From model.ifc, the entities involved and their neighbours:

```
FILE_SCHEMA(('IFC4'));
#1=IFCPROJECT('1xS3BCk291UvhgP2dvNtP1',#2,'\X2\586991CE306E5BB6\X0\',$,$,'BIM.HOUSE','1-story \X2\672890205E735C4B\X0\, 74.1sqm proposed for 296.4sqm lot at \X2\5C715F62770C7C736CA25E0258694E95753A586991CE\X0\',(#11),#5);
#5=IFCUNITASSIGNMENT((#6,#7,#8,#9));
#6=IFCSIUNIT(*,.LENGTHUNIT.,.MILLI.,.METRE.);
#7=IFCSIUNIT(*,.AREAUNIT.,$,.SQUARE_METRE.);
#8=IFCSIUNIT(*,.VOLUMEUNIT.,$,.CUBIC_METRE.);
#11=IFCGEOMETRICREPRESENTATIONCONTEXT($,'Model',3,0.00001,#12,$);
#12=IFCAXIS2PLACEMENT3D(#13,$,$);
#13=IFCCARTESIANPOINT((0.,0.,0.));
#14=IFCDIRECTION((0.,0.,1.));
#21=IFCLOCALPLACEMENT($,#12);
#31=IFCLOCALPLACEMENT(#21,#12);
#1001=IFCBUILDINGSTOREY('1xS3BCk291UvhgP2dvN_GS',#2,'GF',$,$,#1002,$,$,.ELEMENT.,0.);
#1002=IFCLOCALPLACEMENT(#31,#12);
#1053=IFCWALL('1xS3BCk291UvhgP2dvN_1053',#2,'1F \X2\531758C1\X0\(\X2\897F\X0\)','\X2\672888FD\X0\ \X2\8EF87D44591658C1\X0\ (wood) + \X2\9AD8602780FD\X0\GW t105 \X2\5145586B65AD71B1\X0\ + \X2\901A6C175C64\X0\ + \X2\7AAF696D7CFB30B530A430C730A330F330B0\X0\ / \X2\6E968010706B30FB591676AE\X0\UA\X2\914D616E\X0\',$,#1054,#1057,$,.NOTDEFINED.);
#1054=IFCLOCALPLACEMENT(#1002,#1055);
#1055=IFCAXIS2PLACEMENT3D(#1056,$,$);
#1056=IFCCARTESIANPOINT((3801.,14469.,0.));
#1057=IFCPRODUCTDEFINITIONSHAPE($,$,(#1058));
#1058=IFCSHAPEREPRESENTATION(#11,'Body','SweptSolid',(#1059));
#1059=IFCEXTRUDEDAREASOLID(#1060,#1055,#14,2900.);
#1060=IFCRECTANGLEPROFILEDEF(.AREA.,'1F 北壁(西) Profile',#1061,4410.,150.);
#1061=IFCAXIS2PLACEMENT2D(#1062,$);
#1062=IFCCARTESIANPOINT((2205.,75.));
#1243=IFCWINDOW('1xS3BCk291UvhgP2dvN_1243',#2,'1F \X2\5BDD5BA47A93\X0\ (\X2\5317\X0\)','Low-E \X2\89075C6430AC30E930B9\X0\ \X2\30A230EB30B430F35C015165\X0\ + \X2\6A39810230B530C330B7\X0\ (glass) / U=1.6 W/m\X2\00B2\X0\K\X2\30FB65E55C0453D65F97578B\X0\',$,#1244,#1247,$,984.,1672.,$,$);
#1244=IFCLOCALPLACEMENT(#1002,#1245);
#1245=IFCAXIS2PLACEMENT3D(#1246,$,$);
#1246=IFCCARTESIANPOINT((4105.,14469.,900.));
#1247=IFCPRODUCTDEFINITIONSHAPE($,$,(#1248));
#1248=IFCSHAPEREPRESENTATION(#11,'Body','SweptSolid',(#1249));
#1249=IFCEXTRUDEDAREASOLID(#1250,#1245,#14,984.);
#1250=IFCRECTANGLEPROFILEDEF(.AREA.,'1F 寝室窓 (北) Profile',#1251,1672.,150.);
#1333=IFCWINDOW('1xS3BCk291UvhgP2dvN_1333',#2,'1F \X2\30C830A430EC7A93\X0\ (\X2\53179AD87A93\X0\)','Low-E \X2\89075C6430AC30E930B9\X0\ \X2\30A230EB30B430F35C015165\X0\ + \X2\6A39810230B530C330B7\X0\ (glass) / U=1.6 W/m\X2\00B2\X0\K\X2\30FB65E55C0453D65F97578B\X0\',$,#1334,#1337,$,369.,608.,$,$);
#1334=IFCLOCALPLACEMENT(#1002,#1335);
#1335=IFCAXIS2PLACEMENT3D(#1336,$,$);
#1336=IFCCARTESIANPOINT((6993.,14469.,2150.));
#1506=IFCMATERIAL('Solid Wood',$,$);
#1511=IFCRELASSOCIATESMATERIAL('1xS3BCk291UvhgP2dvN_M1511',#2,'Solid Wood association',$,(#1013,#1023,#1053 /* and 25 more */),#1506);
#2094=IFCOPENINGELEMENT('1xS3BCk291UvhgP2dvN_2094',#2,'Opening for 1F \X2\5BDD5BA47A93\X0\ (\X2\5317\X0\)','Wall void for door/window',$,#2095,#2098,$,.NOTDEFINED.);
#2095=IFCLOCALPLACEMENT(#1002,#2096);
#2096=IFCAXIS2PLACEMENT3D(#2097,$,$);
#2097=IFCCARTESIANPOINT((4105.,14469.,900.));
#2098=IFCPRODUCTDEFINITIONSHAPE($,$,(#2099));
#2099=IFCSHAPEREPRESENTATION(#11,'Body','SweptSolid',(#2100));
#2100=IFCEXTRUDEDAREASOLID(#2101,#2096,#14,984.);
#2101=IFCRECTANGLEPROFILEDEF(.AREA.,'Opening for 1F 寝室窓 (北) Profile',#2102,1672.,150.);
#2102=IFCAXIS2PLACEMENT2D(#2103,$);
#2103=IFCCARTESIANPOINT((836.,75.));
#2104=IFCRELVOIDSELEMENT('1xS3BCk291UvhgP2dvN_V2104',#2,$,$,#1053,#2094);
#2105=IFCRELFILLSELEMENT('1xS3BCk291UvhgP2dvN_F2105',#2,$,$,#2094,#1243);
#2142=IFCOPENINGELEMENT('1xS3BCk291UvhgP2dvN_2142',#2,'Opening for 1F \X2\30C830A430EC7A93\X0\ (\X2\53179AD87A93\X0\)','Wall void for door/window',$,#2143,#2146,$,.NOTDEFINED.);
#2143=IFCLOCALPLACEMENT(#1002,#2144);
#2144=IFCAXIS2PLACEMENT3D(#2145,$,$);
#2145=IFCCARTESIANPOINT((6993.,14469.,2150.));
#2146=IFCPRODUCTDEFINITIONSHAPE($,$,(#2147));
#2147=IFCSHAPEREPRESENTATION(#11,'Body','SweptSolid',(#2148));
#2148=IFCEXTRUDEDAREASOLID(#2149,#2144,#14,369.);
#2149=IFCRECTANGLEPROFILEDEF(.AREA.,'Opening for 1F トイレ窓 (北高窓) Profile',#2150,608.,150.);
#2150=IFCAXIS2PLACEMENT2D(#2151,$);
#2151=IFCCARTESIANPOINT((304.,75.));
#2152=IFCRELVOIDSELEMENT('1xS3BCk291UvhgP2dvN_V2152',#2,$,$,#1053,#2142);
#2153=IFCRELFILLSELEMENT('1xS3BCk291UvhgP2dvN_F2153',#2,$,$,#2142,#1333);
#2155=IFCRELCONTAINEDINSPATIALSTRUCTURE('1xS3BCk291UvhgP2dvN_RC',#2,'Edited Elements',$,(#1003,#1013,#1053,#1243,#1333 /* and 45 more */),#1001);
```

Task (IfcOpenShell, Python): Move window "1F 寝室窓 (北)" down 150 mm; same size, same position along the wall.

```python
import numpy as np
import ifcopenshell
import ifcopenshell.api.geometry
import ifcopenshell.util.placement
import ifcopenshell.util.unit

model = ifcopenshell.open("model.ifc")
unit_scale = ifcopenshell.util.unit.calculate_unit_scale(model)

window = model.by_guid("1xS3BCk291UvhgP2dvN_1243")
opening = window.FillsVoids[0].RelatingOpeningElement
dz = -0.15 / unit_scale

shift = np.array([0.0, 0.0, dz])
# The window is not placed relative to its opening, so move both.
for product in (opening, window):
    matrix = ifcopenshell.util.placement.get_local_placement(product.ObjectPlacement)
    matrix[:3, 3] += shift
    ifcopenshell.api.geometry.edit_object_placement(model, product=product, matrix=matrix, is_si=False)

print(f"moved by {dz * unit_scale:+.3f} m")

model.write("model_updated.ifc")
```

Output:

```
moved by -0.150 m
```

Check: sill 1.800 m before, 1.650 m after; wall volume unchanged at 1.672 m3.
